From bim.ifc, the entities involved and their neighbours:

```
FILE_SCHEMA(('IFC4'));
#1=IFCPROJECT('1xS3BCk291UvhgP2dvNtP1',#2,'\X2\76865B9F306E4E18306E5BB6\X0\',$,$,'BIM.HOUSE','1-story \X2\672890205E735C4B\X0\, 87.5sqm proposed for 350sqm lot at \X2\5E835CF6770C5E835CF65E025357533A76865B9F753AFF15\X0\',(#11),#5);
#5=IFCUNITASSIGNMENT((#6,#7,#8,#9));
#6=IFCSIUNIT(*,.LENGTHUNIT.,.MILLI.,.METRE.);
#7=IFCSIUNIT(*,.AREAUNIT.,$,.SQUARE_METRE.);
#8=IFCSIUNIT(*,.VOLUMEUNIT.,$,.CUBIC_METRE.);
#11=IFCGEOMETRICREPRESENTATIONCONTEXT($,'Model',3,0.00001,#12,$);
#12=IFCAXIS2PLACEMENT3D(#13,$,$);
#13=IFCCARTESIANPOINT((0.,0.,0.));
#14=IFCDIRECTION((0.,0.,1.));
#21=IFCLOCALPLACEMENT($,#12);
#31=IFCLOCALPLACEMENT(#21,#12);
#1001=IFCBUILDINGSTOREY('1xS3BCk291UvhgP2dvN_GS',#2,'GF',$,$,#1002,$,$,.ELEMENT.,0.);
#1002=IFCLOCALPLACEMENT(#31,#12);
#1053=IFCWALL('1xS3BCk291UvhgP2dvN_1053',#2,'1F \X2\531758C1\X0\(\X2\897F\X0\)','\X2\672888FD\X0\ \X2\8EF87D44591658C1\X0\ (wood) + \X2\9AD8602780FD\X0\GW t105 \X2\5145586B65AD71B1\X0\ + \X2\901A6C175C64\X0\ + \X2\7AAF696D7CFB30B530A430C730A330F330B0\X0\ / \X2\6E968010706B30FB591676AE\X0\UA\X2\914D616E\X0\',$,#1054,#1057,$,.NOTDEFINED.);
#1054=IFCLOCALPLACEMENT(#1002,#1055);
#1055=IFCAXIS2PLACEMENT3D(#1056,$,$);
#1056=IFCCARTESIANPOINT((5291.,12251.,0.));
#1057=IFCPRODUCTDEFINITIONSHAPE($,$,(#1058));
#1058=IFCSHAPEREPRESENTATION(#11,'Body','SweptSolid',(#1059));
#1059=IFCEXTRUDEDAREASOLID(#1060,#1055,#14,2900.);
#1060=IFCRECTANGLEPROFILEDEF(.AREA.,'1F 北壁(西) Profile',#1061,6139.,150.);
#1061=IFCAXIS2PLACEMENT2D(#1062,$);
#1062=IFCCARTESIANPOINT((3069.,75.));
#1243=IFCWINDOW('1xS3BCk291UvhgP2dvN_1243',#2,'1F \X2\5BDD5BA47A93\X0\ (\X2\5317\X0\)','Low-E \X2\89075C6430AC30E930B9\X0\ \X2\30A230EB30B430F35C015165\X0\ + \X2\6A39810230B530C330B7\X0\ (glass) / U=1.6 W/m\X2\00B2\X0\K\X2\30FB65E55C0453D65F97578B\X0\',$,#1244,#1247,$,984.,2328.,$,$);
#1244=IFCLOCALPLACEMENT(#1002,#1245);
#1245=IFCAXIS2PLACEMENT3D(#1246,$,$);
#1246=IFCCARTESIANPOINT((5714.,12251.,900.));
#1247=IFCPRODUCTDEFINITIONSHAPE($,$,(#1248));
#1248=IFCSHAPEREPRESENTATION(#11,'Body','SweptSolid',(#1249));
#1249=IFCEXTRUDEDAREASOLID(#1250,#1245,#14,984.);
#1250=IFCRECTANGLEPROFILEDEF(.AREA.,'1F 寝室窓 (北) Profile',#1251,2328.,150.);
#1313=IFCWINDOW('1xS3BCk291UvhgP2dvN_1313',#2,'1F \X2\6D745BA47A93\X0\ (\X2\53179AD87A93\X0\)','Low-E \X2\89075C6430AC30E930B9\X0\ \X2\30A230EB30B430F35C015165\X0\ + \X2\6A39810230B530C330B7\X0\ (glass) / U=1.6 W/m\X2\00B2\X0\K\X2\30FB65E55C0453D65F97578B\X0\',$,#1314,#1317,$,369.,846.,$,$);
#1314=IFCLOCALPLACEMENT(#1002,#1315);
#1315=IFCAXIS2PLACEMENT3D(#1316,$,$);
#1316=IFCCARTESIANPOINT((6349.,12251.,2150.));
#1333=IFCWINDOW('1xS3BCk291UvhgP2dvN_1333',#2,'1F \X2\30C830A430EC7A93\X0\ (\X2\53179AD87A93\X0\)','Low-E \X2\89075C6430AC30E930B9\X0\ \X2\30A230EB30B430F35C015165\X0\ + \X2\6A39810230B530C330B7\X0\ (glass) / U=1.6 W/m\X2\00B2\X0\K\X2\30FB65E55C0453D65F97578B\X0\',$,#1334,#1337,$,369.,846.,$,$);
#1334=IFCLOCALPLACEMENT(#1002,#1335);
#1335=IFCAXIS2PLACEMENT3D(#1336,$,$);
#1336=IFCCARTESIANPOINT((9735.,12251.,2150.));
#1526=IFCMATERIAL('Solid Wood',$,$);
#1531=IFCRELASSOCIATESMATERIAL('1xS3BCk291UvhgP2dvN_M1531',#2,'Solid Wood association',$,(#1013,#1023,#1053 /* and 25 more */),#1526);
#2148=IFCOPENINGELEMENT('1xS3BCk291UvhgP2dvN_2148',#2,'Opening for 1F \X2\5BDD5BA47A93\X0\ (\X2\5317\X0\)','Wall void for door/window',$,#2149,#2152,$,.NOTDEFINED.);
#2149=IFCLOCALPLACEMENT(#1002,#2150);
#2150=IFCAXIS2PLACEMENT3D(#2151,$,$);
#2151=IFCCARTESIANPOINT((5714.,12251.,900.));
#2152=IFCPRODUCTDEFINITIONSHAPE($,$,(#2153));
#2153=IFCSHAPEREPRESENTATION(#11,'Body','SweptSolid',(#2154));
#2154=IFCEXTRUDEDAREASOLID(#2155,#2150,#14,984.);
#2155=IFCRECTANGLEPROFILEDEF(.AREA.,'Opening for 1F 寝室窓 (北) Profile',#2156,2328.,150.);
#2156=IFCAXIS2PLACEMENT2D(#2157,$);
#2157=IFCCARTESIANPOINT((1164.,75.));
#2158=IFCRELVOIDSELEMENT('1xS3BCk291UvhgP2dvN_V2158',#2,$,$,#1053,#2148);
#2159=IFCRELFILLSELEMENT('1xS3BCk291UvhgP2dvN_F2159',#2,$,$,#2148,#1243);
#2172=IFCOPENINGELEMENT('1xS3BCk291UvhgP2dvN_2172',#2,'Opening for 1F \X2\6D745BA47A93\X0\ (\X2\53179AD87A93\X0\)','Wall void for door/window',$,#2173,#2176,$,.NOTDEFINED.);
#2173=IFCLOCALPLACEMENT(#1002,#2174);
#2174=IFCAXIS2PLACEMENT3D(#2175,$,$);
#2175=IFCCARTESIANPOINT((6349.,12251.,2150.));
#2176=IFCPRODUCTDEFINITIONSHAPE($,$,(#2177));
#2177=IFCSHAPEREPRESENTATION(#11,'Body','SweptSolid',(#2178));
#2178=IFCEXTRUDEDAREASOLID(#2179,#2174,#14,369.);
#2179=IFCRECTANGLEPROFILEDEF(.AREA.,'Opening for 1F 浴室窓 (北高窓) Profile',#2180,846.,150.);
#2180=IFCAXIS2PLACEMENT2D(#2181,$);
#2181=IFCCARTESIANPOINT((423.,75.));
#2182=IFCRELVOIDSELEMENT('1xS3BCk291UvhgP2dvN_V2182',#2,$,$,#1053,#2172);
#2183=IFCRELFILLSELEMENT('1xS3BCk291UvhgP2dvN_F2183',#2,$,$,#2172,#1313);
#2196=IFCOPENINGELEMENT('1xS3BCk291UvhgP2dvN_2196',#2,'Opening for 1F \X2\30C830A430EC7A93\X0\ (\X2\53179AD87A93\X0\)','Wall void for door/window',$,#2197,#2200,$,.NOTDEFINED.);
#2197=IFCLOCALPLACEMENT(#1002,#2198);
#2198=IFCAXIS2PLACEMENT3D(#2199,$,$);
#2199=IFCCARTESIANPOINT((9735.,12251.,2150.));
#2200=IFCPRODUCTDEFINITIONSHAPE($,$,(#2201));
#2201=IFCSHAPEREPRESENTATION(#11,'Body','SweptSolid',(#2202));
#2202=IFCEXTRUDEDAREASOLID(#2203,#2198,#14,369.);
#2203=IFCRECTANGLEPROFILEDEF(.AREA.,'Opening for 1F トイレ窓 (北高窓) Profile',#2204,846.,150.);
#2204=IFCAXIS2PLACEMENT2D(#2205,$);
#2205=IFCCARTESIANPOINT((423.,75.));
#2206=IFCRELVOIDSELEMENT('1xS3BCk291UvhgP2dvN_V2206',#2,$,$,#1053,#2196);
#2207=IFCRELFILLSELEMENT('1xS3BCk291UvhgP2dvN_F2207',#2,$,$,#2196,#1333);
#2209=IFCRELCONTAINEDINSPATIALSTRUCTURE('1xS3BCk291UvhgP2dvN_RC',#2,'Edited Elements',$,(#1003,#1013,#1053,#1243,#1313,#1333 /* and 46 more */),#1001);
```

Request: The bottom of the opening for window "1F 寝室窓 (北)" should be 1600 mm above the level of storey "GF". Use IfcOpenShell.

```python
import numpy as np
import ifcopenshell
import ifcopenshell.api.geometry
import ifcopenshell.geom
import ifcopenshell.util.element
import ifcopenshell.util.placement
import ifcopenshell.util.shape
import ifcopenshell.util.unit

model = ifcopenshell.open("bim.ifc")
unit_scale = ifcopenshell.util.unit.calculate_unit_scale(model)

window = model.by_guid("1xS3BCk291UvhgP2dvN_1243")
opening = window.FillsVoids[0].RelatingOpeningElement
storey = ifcopenshell.util.element.get_container(window, ifc_class="IfcBuildingStorey")
level = ifcopenshell.util.placement.get_local_placement(storey.ObjectPlacement)[2, 3]

# The opening's origin need not be at the sill, so measure its lowest point.
shape = ifcopenshell.geom.create_shape(ifcopenshell.geom.settings(), opening)
bottom = ifcopenshell.util.shape.get_shape_bottom_elevation(shape, shape.geometry) / unit_scale
dz = level + 1.6 / unit_scale - bottom

shift = np.array([0.0, 0.0, dz])
# The window is not placed relative to its opening, so move both.
for product in (opening, window):
    matrix = ifcopenshell.util.placement.get_local_placement(product.ObjectPlacement)
    matrix[:3, 3] += shift
    ifcopenshell.api.geometry.edit_object_placement(model, product=product, matrix=matrix, is_si=False)

print(f"moved by {dz * unit_scale:+.3f} m")

model.write("bim_edited.ifc")
```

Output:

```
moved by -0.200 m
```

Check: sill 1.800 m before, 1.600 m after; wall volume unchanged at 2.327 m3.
